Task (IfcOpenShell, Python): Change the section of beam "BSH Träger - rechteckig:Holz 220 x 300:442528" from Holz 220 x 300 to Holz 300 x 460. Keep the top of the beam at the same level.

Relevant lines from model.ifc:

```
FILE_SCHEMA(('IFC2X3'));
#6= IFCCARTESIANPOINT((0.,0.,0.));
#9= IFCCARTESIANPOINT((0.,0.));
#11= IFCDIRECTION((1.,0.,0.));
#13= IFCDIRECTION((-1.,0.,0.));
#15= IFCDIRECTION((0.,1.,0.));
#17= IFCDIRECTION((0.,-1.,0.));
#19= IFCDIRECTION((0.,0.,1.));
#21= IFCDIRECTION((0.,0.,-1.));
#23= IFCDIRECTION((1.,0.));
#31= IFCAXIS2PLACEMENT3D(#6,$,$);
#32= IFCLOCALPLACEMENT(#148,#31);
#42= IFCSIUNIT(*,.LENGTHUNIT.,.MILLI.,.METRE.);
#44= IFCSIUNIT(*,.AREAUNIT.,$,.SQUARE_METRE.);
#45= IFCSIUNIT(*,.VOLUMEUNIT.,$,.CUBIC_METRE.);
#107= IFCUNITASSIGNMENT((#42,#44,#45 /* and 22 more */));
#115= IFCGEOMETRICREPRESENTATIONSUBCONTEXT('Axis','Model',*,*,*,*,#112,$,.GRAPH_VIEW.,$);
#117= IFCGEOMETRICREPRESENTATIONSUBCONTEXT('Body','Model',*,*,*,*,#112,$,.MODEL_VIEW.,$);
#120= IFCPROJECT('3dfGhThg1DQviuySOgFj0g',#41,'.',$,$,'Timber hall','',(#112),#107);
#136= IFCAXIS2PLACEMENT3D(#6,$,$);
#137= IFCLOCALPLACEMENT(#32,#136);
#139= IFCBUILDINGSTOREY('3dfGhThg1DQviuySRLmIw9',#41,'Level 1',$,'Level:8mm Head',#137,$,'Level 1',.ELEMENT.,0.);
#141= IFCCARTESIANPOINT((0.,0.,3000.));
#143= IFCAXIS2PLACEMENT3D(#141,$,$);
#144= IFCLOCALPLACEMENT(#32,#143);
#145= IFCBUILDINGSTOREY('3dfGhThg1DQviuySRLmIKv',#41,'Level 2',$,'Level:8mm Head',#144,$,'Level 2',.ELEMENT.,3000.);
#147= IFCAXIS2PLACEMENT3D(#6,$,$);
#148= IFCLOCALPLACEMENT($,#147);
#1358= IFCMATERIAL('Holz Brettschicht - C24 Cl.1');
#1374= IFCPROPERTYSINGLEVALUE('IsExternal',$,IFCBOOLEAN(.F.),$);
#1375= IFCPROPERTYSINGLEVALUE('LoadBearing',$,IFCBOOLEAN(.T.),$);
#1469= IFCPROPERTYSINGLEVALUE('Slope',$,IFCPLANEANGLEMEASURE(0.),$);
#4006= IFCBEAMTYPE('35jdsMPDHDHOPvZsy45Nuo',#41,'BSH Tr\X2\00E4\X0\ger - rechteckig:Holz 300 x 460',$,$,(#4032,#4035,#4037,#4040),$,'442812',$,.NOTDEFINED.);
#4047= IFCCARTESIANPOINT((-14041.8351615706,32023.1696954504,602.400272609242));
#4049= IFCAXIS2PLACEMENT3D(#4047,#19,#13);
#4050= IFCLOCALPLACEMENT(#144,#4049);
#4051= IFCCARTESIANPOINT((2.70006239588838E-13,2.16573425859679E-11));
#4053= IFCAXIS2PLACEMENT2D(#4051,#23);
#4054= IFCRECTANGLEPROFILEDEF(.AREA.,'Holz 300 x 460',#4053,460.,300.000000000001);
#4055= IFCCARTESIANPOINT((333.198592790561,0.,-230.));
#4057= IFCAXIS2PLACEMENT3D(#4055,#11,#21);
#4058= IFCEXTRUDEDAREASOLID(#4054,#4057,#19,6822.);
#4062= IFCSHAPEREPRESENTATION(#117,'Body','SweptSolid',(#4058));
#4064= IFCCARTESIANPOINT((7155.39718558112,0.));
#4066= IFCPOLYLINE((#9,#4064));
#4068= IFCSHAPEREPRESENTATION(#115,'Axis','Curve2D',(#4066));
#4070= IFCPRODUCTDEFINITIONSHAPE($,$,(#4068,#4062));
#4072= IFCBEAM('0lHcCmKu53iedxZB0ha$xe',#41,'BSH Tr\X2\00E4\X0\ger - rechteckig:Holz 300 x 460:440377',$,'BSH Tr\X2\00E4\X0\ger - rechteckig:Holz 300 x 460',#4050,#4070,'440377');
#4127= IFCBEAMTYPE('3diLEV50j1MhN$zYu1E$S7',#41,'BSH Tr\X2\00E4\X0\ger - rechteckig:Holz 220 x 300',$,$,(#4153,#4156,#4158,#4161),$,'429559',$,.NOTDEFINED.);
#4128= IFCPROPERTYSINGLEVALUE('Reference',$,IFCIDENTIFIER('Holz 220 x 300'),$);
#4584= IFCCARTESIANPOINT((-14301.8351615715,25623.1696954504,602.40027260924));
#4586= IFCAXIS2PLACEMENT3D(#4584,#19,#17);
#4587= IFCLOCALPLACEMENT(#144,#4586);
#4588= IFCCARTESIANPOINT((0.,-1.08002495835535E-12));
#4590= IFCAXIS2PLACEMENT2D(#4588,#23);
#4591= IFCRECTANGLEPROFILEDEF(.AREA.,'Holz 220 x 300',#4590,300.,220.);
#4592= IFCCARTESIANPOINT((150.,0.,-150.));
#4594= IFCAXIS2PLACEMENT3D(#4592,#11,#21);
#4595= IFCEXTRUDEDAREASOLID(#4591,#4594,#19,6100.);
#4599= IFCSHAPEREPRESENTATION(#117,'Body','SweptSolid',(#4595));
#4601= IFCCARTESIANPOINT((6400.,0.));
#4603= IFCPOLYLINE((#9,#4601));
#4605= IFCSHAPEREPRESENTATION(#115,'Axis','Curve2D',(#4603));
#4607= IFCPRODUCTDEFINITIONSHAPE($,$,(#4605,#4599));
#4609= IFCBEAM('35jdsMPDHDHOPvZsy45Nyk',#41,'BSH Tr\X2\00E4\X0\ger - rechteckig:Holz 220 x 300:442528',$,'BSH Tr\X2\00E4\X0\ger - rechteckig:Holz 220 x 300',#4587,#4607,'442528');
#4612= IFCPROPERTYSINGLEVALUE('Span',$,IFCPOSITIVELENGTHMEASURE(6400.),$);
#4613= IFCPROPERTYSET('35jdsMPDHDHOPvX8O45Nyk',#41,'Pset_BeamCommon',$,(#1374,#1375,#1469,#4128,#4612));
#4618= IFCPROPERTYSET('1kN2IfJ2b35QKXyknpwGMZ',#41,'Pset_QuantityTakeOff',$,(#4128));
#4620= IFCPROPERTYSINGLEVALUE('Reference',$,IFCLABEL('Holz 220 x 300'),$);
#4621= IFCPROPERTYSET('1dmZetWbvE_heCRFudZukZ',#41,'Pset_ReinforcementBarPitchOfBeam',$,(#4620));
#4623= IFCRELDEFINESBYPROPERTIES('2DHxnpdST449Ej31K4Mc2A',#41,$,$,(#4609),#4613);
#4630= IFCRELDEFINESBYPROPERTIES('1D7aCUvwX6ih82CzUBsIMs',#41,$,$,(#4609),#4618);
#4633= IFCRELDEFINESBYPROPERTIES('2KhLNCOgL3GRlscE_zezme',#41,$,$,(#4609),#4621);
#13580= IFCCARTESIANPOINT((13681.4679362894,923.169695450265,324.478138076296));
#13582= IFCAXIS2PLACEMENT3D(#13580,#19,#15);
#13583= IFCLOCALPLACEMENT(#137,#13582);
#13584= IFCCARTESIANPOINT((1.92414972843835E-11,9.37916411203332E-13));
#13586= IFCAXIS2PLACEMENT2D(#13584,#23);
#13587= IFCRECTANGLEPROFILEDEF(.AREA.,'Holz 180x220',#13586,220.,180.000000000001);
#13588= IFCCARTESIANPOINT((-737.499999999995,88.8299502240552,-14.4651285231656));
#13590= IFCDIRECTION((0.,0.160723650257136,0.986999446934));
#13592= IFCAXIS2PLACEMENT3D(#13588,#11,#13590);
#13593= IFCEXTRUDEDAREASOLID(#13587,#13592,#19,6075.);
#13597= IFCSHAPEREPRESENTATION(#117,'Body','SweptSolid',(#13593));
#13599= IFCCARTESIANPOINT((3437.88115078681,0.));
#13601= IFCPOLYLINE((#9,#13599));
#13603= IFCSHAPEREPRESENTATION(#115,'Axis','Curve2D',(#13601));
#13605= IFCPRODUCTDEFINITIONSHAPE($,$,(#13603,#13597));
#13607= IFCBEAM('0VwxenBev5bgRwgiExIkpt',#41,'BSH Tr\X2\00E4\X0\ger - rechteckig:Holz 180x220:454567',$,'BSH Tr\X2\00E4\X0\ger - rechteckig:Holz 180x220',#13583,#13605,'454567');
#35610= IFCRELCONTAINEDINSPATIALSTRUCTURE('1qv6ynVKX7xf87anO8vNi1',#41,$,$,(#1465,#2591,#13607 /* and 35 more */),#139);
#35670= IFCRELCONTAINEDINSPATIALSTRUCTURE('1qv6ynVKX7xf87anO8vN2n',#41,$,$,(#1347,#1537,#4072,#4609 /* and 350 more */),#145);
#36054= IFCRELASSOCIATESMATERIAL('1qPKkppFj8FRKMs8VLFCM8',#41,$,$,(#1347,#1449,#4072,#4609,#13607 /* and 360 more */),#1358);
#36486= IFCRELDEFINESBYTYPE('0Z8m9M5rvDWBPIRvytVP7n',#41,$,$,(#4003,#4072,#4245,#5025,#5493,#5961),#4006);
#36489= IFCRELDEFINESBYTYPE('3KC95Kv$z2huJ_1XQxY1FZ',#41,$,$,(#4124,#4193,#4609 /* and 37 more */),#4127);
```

```python
import ifcopenshell
import ifcopenshell.api.pset
import ifcopenshell.api.type
import ifcopenshell.util.element
import ifcopenshell.util.representation

model = ifcopenshell.open("model.ifc")

member = model.by_id(4609)
source = next(p for p in model.by_type("IfcRectangleProfileDef") if p.ProfileName == "Holz 300 x 460")

body = ifcopenshell.util.representation.get_representation(member, "Model", "Body")
solid = body.Items[0]
old_profile = solid.SweptArea

# Copy the section's sizes but keep this member's own profile position.
profile = ifcopenshell.util.element.copy(model, source)
# Profiles are centred, so shift by half the change in depth to hold the top.
shift = (old_profile.XDim - profile.XDim) / 2
x, y = old_profile.Position.Location.Coordinates
up = (-1.0, 0.0)  # upwards, in the solid's own plane
location = model.createIfcCartesianPoint((x + up[0] * shift, y + up[1] * shift))
profile.Position = model.createIfcAxis2Placement2D(location, old_profile.Position.RefDirection)
solid.SweptArea = profile
if not model.get_total_inverses(old_profile):
    ifcopenshell.util.element.remove_deep2(model, old_profile)

new_type = model.by_id(4006)
ifcopenshell.api.type.assign_type(
    model, related_objects=[member], relating_type=new_type, should_map_representations=False
)
member.Name = member.Name.replace("Holz 220 x 300", "Holz 300 x 460")
member.ObjectType = "BSH Träger - rechteckig:Holz 300 x 460"
pset = model.by_id(ifcopenshell.util.element.get_pset(member, "Pset_BeamCommon", should_inherit=False)["id"])
ifcopenshell.api.pset.edit_pset(model, pset=pset, properties={"Reference": "Holz 300 x 460"})
pset = model.by_id(ifcopenshell.util.element.get_pset(member, "Pset_QuantityTakeOff", should_inherit=False)["id"])
ifcopenshell.api.pset.edit_pset(model, pset=pset, properties={"Reference": "Holz 300 x 460"})
pset = model.by_id(ifcopenshell.util.element.get_pset(member, "Pset_ReinforcementBarPitchOfBeam", should_inherit=False)["id"])
ifcopenshell.api.pset.edit_pset(model, pset=pset, properties={"Reference": "Holz 300 x 460"})

print(solid.SweptArea)

model.write("model_updated.ifc")
```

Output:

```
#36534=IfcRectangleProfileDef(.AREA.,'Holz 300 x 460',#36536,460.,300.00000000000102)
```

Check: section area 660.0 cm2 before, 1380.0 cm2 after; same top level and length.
